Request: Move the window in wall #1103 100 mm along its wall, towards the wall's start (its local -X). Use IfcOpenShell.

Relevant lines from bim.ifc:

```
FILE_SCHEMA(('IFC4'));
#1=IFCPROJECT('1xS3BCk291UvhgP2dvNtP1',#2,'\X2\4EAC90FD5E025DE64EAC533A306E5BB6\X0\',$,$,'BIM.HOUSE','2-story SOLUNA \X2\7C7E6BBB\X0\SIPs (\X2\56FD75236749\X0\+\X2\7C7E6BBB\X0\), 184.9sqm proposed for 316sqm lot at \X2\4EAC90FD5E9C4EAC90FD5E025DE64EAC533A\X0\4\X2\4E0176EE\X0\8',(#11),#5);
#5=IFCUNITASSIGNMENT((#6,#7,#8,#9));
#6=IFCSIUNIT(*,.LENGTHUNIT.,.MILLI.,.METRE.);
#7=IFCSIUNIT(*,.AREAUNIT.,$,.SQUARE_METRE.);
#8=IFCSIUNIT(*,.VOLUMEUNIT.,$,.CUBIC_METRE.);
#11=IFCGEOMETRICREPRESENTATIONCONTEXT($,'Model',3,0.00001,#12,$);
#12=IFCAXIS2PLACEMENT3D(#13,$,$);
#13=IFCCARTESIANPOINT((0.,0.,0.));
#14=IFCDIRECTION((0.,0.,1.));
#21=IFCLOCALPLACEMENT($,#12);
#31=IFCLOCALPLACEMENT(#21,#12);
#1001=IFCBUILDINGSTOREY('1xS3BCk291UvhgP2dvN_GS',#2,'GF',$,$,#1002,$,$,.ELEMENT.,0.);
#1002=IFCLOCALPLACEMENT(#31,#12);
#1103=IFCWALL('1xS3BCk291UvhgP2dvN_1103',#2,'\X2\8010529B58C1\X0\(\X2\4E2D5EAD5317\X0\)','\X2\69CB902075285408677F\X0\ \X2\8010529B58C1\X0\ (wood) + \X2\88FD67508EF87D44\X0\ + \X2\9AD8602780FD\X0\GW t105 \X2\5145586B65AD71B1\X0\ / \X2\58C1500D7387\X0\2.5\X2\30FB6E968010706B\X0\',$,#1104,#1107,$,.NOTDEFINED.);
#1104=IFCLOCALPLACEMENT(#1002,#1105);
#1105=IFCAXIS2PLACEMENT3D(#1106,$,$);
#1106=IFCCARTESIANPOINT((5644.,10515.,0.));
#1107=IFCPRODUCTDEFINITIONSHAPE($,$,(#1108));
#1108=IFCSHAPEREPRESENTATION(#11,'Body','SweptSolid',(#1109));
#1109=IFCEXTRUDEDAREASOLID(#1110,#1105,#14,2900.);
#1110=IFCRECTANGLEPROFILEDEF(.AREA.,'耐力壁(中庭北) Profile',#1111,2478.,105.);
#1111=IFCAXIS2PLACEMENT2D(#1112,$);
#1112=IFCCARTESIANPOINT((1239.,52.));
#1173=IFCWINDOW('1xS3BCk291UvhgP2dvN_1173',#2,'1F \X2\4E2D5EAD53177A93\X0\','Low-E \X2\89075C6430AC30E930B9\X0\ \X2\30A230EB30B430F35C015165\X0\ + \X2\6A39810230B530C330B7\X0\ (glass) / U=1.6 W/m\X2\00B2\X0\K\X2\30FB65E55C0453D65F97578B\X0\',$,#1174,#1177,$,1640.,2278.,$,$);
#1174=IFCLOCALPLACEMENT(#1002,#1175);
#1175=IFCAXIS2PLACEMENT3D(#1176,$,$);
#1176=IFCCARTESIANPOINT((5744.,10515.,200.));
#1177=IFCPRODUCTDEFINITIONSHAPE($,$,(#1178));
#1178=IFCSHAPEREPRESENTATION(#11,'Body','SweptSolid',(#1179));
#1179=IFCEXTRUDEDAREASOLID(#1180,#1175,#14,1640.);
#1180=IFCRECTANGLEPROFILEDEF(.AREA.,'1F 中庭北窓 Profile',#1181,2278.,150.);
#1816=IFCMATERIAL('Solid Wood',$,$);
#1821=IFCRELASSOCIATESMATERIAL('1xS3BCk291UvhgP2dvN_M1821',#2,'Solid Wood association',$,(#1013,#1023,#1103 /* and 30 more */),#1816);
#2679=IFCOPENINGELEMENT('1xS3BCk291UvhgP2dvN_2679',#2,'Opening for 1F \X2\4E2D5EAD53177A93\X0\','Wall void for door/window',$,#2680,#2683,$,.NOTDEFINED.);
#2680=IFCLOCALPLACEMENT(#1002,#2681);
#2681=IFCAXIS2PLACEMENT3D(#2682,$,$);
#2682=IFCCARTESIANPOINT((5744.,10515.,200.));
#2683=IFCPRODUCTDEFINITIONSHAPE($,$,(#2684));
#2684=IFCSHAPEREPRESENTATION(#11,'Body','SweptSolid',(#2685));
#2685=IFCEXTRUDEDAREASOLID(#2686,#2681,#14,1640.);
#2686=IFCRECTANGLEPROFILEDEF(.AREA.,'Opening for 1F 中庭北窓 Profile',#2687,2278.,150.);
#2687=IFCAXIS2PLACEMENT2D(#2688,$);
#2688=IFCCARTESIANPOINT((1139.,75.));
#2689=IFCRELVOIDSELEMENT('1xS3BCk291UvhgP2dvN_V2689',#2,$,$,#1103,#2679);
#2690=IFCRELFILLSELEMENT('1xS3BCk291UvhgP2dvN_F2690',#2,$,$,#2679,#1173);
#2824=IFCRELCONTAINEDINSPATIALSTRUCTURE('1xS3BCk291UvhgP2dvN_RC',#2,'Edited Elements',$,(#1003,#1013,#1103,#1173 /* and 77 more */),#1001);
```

```python
import ifcopenshell
import ifcopenshell.api.geometry
import ifcopenshell.util.placement
import ifcopenshell.util.unit

model = ifcopenshell.open("bim.ifc")
unit_scale = ifcopenshell.util.unit.calculate_unit_scale(model)

window = model.by_guid("1xS3BCk291UvhgP2dvN_1173")
opening = window.FillsVoids[0].RelatingOpeningElement
wall = opening.VoidsElements[0].RelatingBuildingElement

wall_matrix = ifcopenshell.util.placement.get_local_placement(wall.ObjectPlacement)
shift = wall_matrix[:3, 0] * -0.1 / unit_scale
before = ifcopenshell.util.placement.get_local_placement(window.ObjectPlacement)[:3, 3].copy()

# The window is not placed relative to its opening, so move both.
for product in (opening, window):
    matrix = ifcopenshell.util.placement.get_local_placement(product.ObjectPlacement)
    matrix[:3, 3] += shift
    ifcopenshell.api.geometry.edit_object_placement(model, product=product, matrix=matrix, is_si=False)

after = ifcopenshell.util.placement.get_local_placement(window.ObjectPlacement)[:3, 3]
print("window moved by", (after - before).round(3) + 0.0)

model.write("bim_v2.ifc")
```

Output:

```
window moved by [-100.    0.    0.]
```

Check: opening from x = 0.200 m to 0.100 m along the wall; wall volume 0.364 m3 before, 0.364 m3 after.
